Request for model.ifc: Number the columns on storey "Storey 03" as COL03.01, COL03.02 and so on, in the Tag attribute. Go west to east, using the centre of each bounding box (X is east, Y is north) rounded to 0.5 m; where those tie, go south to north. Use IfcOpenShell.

First a look at what the model holds.

```python
import ifcopenshell
import ifcopenshell.util.element
import ifcopenshell.util.placement

model = ifcopenshell.open("model.ifc")
print(model.schema)
storey = next(s for s in model.by_type("IfcBuildingStorey") if s.Name == "Storey 03")
columns = [e for e in ifcopenshell.util.element.get_decomposition(storey) if e.is_a("IfcColumn")]
for e in sorted(columns, key=lambda e: e.id()):
    origin = ifcopenshell.util.placement.get_local_placement(e.ObjectPlacement)[:3, 3]
    print(e.id(), e.Tag, e.Name, origin.round(2) + 0.0, sep=" | ")
```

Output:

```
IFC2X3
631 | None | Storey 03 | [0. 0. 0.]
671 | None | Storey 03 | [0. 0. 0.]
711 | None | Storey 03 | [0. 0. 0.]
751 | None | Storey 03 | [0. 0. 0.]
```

```python
import ifcopenshell
import ifcopenshell.geom
import ifcopenshell.util.element
import ifcopenshell.util.shape

model = ifcopenshell.open("model.ifc")
settings = ifcopenshell.geom.settings()
settings.set("use-world-coords", True)


def centre(element):
    shape = ifcopenshell.geom.create_shape(settings, element)
    return ifcopenshell.util.shape.get_bbox_centroid(shape.geometry)


storey = next(s for s in model.by_type("IfcBuildingStorey") if s.Name == "Storey 03")
columns = [e for e in ifcopenshell.util.element.get_decomposition(storey) if e.is_a("IfcColumn")]

# Insertion points can sit at a corner or the storey origin, so sort by the geometry (in metres).
centres = {e: centre(e) for e in columns}
columns.sort(key=lambda e: (round(centres[e][0] / 0.5), centres[e][1]))

for i, e in enumerate(columns, start=1):
    number = f"COL03.{i:02d}"
    e.Tag = number
    print(e.id(), number)

model.write("model_v2.ifc")
```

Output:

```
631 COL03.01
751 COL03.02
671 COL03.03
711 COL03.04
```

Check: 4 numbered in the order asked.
